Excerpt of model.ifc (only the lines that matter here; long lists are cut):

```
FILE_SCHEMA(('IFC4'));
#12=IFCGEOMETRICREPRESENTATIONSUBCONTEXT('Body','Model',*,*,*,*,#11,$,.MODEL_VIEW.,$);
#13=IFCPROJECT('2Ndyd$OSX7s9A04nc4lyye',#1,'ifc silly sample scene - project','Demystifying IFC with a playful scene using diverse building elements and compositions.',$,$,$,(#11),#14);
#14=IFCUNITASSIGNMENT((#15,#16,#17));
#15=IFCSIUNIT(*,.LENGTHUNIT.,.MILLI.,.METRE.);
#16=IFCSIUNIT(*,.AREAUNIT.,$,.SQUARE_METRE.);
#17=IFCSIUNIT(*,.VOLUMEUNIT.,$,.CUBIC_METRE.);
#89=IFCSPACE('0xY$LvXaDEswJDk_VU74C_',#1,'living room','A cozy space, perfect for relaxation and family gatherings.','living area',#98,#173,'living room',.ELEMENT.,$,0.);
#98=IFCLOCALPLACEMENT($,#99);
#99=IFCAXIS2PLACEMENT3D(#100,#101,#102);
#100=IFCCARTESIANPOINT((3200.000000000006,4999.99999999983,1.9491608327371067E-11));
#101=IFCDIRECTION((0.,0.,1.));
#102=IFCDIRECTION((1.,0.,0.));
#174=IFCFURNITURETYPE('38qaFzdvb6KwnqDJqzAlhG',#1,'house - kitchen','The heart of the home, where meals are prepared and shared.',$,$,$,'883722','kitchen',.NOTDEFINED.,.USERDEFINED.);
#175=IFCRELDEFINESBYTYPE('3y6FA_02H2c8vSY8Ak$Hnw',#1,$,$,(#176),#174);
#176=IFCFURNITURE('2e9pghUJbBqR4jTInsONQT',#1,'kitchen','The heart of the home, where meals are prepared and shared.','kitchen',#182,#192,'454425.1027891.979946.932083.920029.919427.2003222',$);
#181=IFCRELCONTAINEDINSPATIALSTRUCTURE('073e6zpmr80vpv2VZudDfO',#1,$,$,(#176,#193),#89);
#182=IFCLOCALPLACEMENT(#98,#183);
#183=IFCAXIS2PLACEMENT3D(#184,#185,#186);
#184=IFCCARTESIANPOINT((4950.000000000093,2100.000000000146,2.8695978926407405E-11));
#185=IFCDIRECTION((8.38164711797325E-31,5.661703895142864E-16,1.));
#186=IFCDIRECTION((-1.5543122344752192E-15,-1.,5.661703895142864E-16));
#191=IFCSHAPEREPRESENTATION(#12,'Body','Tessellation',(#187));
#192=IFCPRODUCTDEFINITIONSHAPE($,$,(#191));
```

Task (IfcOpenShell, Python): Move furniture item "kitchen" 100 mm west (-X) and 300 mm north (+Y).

```python
import ifcopenshell
import ifcopenshell.api.geometry
import ifcopenshell.util.placement
import ifcopenshell.util.unit

model = ifcopenshell.open("model.ifc")
unit_scale = ifcopenshell.util.unit.calculate_unit_scale(model)

item = model.by_guid("2e9pghUJbBqR4jTInsONQT")
matrix = ifcopenshell.util.placement.get_local_placement(item.ObjectPlacement)
matrix[0, 3] -= 0.1 / unit_scale
matrix[1, 3] += 0.3 / unit_scale
ifcopenshell.api.geometry.edit_object_placement(model, product=item, matrix=matrix, is_si=False)

print(ifcopenshell.util.placement.get_local_placement(item.ObjectPlacement).round(3) + 0.0)

model.write("model-out.ifc")
```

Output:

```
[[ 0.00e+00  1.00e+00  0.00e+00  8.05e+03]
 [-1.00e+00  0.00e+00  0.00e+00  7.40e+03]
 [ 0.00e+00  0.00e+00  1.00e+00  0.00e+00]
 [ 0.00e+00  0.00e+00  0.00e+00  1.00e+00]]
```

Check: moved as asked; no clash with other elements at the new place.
